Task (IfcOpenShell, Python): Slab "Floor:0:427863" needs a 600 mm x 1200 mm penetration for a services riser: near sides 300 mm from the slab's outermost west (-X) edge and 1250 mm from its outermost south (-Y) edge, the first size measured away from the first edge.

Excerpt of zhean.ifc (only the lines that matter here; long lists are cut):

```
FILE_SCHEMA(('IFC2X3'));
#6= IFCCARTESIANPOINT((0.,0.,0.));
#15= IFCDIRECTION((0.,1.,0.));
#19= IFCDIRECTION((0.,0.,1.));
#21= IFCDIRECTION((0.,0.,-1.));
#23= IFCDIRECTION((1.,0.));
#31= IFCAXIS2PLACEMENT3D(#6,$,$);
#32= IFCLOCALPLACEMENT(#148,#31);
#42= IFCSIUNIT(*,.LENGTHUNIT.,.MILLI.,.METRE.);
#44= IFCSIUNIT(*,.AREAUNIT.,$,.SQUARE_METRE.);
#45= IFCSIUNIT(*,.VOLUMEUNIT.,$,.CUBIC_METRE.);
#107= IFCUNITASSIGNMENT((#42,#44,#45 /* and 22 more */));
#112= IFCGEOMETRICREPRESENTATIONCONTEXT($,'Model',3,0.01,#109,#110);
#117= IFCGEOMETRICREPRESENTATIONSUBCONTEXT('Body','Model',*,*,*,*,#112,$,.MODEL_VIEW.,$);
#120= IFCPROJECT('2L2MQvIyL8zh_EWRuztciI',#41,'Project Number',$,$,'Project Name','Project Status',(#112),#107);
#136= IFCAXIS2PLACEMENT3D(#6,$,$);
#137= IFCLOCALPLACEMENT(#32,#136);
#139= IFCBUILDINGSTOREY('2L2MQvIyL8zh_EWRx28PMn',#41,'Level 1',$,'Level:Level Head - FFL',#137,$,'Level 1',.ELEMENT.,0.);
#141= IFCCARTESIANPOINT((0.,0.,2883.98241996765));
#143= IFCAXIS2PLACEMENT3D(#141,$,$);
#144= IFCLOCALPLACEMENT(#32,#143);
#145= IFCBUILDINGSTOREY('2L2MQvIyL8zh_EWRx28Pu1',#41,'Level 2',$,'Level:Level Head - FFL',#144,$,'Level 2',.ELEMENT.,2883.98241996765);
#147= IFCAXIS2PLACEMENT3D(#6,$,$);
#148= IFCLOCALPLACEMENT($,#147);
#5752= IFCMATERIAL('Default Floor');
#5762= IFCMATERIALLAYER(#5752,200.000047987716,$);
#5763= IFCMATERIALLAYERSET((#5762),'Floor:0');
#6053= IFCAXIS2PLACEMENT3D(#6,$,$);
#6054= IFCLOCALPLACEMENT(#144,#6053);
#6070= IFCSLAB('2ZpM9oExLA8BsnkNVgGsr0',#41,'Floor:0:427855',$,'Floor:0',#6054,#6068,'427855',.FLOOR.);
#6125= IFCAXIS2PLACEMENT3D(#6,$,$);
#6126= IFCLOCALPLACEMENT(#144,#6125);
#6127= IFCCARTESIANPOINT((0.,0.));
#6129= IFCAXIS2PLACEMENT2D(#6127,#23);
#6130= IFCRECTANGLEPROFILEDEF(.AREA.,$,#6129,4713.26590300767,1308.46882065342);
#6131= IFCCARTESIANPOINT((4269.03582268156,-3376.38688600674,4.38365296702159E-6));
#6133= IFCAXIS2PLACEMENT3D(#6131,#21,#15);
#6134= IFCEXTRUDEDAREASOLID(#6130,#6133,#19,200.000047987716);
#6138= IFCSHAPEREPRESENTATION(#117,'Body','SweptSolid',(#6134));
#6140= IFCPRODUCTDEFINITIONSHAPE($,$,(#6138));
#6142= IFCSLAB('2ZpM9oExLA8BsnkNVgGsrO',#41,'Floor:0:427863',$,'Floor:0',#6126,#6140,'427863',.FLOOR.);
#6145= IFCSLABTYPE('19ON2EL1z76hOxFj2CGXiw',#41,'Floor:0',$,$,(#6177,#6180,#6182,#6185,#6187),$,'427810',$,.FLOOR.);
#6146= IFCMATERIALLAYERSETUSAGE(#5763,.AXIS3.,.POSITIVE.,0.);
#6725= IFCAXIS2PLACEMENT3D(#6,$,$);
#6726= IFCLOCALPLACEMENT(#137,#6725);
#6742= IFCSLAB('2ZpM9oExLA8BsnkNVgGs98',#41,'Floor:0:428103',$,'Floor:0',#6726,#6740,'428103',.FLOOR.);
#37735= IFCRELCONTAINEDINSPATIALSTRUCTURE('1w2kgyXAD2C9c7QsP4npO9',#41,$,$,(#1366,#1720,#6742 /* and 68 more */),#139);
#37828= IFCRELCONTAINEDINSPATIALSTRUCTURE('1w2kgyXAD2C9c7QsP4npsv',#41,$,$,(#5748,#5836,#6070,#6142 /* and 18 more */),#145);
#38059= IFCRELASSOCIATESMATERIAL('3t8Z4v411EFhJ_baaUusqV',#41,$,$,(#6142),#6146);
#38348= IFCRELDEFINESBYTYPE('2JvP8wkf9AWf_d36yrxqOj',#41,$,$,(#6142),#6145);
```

```python
import numpy as np
import ifcopenshell
import ifcopenshell.api.feature
import ifcopenshell.api.geometry
import ifcopenshell.api.root
import ifcopenshell.geom
import ifcopenshell.util.placement
import ifcopenshell.util.representation
import ifcopenshell.util.shape
import ifcopenshell.util.unit

model = ifcopenshell.open("zhean.ifc")
unit_scale = ifcopenshell.util.unit.calculate_unit_scale(model)
settings = ifcopenshell.geom.settings()


def volume(element):
    """Net volume in cubic metres, openings subtracted."""
    shape = ifcopenshell.geom.create_shape(settings, element)
    return ifcopenshell.util.shape.get_volume(shape.geometry)


slab = model.by_id(6142)
before = volume(slab)

# Extent in the slab's own axes, in metres. The edges named are its -X and -Y sides.
slab_shape = ifcopenshell.geom.create_shape(settings, slab)
vertices = ifcopenshell.util.shape.get_vertices(slab_shape.geometry)
x_min, y_min, bottom = vertices.min(axis=0)
top = vertices[:, 2].max()

opening = ifcopenshell.api.root.create_entity(model, ifc_class="IfcOpeningElement", name="Services riser opening")
context = ifcopenshell.util.representation.get_context(model, "Model", "Body", "MODEL_VIEW")
width, depth = 0.6, 1.2
outline = [(0.0, 0.0), (width, 0.0), (width, depth), (0.0, depth), (0.0, 0.0)]
# Overshoot both faces by 50 mm so the cut is clean.
shape = ifcopenshell.api.geometry.add_slab_representation(
    model, context=context, depth=top - bottom + 0.1, polyline=outline
)
ifcopenshell.api.geometry.assign_representation(model, product=opening, representation=shape)

matrix = ifcopenshell.util.placement.get_local_placement(slab.ObjectPlacement)
matrix[:, 3] = matrix @ np.append(np.array([x_min + 0.3, y_min + 1.25, bottom - 0.05]) / unit_scale, 1.0)
ifcopenshell.api.geometry.edit_object_placement(model, product=opening, matrix=matrix, is_si=False)
ifcopenshell.api.feature.add_feature(model, feature=opening, element=slab)

after = volume(slab)

print(f"slab volume {before:.3f} -> {after:.3f} m3")

model.write("zhean-out.ifc")
```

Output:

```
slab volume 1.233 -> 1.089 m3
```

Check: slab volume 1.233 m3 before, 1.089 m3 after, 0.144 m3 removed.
